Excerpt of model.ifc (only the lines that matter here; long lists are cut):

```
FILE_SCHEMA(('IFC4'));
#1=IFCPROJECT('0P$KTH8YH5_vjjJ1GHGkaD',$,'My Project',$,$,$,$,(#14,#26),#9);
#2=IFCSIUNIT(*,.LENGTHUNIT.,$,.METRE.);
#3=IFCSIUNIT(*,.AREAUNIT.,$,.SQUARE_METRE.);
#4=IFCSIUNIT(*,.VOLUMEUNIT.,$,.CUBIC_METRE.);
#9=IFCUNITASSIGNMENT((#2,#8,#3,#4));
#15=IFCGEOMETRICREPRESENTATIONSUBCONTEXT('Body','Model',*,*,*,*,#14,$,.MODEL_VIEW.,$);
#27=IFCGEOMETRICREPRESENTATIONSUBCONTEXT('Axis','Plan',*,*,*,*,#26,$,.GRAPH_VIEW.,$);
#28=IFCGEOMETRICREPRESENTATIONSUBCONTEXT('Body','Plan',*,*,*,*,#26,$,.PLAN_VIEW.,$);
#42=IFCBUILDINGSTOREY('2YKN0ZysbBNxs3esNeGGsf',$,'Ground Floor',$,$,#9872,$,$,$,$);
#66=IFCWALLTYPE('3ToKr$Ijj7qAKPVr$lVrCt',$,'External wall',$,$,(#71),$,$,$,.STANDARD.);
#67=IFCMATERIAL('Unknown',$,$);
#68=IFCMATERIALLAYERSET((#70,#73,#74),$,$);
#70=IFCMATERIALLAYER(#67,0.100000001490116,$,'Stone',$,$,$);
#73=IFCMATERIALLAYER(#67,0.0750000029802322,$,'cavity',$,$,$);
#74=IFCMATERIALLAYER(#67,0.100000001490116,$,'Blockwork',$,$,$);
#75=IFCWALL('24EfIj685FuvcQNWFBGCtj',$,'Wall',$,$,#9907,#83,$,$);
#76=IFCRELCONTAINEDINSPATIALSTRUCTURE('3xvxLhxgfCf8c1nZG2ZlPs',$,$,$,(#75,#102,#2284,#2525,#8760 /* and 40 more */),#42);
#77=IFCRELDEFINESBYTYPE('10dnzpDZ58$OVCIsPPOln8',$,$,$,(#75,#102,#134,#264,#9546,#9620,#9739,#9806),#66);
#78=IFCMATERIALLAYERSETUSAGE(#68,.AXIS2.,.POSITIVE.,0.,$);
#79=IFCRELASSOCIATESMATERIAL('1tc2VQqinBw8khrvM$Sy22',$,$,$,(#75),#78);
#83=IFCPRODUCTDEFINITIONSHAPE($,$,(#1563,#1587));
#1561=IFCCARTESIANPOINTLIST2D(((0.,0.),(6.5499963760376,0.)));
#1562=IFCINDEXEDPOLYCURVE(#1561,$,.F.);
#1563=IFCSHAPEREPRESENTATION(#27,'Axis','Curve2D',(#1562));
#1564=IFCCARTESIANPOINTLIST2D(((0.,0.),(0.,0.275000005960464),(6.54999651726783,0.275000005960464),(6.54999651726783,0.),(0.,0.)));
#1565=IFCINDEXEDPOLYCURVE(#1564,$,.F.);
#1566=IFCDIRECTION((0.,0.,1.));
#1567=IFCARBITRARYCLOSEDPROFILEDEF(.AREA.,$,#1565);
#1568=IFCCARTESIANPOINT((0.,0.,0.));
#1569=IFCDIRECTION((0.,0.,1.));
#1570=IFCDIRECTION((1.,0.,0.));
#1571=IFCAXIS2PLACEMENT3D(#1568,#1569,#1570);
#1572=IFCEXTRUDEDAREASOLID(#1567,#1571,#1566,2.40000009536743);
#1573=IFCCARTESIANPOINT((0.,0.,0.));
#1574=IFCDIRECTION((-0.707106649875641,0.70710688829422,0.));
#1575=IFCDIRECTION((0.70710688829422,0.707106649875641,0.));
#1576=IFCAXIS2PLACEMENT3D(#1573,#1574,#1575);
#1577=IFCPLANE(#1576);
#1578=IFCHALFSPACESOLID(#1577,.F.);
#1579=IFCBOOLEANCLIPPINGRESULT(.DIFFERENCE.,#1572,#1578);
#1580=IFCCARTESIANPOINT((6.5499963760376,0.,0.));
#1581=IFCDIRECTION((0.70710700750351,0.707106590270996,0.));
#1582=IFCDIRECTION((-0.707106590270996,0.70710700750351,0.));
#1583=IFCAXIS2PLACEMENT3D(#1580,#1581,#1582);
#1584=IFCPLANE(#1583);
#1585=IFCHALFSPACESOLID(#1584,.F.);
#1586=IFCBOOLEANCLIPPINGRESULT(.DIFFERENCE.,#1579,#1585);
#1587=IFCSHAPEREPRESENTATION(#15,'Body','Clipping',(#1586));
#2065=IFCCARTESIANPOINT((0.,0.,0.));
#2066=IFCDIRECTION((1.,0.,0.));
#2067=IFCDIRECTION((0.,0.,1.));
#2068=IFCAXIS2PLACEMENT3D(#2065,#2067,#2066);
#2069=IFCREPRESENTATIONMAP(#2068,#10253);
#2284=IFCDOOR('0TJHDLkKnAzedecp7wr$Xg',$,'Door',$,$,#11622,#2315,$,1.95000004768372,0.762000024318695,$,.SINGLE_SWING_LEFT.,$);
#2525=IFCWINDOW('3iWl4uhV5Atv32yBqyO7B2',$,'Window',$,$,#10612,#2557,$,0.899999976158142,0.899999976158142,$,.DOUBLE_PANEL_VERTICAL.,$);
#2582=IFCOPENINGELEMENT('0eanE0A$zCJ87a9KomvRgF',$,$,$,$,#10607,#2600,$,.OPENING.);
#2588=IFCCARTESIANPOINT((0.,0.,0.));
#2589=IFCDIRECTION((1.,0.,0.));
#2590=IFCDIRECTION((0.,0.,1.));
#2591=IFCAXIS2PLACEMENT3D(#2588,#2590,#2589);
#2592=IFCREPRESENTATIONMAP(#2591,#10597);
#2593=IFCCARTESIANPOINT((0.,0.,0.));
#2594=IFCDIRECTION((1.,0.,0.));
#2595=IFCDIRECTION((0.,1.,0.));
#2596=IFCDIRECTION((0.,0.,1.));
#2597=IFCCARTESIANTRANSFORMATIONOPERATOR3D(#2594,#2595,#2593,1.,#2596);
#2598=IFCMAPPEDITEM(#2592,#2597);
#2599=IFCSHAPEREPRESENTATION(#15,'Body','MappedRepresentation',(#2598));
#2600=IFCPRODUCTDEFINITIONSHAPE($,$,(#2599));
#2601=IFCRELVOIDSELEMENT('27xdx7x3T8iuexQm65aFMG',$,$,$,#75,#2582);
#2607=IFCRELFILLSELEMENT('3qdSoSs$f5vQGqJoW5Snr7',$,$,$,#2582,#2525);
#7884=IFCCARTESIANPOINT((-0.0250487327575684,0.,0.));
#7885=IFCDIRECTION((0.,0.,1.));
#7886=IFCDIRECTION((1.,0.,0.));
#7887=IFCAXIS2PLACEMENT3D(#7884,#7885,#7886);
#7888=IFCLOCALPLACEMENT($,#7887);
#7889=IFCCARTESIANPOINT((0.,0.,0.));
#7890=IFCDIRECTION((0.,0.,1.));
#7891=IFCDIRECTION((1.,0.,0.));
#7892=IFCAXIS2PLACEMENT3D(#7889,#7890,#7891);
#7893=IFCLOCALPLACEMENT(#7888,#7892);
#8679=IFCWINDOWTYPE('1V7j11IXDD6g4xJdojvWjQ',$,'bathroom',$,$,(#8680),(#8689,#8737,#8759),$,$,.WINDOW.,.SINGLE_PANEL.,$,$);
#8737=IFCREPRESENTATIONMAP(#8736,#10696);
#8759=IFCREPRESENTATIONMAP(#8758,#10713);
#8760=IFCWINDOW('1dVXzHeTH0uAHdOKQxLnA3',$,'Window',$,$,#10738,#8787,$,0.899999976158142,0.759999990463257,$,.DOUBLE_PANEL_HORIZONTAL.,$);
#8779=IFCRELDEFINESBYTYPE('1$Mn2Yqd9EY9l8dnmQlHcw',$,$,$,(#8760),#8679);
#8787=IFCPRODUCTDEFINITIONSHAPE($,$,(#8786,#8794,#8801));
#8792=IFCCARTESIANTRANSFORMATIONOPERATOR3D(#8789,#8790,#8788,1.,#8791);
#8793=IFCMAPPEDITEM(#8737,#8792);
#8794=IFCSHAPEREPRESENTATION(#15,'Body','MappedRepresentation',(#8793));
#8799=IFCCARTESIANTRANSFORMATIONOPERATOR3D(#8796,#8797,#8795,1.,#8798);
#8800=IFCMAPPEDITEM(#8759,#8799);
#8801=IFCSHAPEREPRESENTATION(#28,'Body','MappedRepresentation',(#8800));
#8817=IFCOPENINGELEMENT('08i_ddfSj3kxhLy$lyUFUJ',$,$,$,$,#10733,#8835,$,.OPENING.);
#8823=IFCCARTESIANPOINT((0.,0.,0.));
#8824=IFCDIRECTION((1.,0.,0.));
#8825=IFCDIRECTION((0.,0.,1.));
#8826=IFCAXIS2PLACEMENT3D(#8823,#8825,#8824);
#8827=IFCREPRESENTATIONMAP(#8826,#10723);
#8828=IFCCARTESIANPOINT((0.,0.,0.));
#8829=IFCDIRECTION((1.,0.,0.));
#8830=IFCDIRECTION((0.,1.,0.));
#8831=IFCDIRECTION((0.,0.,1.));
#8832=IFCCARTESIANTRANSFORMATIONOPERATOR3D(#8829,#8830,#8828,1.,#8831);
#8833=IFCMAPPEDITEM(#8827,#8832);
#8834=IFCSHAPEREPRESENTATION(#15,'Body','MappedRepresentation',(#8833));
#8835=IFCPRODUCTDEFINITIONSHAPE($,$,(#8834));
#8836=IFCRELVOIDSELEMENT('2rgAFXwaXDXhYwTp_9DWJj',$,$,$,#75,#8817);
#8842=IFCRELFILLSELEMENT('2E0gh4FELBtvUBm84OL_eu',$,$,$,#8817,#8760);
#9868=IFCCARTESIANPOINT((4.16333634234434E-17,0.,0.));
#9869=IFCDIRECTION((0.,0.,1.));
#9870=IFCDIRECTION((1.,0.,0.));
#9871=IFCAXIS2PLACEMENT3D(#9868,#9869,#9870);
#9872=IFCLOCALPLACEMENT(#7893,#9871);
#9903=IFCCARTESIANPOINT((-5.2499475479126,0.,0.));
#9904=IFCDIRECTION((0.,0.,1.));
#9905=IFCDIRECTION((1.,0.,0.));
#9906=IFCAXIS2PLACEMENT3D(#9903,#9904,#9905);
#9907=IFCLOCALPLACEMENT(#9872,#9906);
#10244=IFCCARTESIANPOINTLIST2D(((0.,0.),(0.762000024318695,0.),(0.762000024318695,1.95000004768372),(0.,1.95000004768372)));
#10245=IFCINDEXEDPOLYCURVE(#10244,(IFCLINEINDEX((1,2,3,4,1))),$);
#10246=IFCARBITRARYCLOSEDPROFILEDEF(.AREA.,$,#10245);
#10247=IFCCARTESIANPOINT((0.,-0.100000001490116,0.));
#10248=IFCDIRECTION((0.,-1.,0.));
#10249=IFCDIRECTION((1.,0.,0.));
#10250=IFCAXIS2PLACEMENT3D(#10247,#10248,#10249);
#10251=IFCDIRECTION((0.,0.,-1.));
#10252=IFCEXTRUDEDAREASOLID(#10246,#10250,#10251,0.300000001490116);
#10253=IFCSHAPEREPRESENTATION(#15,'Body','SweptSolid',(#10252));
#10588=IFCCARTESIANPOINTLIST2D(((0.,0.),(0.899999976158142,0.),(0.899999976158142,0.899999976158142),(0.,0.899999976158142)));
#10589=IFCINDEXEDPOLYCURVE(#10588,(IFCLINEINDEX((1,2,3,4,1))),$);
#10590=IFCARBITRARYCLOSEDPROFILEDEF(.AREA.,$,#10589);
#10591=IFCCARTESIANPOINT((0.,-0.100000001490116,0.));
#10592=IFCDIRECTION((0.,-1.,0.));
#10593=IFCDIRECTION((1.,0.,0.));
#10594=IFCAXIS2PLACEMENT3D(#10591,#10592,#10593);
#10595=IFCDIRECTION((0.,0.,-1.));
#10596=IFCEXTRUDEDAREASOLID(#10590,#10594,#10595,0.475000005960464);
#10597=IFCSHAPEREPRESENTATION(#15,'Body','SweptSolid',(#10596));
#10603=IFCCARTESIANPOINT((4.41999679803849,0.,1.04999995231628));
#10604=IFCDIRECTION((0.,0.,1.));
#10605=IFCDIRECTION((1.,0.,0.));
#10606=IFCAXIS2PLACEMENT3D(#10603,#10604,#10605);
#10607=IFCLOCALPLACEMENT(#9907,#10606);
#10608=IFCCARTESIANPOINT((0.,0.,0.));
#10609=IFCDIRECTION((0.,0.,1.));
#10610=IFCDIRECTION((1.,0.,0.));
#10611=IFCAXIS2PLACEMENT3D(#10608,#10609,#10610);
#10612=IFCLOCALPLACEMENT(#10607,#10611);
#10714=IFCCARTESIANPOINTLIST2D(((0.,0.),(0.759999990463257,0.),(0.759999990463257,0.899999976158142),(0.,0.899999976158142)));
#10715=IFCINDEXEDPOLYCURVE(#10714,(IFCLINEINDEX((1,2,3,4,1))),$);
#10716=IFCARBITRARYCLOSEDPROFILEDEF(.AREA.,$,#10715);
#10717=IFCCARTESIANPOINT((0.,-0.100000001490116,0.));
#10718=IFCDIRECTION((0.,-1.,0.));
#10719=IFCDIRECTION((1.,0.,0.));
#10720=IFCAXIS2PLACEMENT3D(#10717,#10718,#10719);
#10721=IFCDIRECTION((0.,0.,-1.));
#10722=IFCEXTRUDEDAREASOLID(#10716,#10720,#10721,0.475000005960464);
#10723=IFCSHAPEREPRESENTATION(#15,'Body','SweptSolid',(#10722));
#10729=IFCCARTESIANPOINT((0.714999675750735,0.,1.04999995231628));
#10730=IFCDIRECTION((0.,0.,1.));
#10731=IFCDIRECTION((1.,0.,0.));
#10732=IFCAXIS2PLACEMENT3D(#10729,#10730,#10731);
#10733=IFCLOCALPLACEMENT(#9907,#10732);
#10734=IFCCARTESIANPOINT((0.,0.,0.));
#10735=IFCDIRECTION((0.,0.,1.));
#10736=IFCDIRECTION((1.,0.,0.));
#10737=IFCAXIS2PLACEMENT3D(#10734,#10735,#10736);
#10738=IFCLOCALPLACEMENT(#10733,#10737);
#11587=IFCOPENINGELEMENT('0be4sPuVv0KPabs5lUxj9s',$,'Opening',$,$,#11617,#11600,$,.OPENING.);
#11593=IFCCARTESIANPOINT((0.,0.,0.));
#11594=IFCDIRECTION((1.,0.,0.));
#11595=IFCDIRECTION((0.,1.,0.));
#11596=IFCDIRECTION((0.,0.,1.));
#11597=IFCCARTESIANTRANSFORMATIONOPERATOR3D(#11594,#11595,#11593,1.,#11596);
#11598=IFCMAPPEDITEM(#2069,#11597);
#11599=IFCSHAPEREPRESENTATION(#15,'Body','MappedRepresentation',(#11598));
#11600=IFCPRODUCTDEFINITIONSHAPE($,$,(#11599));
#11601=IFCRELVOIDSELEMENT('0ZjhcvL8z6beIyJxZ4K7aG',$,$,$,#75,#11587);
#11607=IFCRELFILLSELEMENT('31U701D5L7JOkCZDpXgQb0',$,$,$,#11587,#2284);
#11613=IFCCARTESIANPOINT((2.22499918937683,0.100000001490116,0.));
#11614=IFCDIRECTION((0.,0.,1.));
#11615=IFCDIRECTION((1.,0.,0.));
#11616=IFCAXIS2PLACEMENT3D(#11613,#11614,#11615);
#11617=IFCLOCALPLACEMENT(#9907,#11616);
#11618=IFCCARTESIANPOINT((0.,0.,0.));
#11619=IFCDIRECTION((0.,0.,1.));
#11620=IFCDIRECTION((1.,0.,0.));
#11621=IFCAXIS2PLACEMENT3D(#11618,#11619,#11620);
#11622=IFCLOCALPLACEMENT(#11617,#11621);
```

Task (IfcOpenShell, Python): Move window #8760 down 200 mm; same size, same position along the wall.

```python
import numpy as np
import ifcopenshell
import ifcopenshell.api.geometry
import ifcopenshell.util.placement
import ifcopenshell.util.unit

model = ifcopenshell.open("model.ifc")
unit_scale = ifcopenshell.util.unit.calculate_unit_scale(model)

window = model.by_id(8760)
opening = window.FillsVoids[0].RelatingOpeningElement
dz = -0.2 / unit_scale

shift = np.array([0.0, 0.0, dz])
# The window is placed relative to its opening, so it follows when the opening moves.
matrix = ifcopenshell.util.placement.get_local_placement(opening.ObjectPlacement)
matrix[:3, 3] += shift
ifcopenshell.api.geometry.edit_object_placement(
    model, product=opening, matrix=matrix, is_si=False, should_transform_children=True
)

print(f"moved by {dz * unit_scale:+.3f} m")

model.write("model_v2.ifc")
```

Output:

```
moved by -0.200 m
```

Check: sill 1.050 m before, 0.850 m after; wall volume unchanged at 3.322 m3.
